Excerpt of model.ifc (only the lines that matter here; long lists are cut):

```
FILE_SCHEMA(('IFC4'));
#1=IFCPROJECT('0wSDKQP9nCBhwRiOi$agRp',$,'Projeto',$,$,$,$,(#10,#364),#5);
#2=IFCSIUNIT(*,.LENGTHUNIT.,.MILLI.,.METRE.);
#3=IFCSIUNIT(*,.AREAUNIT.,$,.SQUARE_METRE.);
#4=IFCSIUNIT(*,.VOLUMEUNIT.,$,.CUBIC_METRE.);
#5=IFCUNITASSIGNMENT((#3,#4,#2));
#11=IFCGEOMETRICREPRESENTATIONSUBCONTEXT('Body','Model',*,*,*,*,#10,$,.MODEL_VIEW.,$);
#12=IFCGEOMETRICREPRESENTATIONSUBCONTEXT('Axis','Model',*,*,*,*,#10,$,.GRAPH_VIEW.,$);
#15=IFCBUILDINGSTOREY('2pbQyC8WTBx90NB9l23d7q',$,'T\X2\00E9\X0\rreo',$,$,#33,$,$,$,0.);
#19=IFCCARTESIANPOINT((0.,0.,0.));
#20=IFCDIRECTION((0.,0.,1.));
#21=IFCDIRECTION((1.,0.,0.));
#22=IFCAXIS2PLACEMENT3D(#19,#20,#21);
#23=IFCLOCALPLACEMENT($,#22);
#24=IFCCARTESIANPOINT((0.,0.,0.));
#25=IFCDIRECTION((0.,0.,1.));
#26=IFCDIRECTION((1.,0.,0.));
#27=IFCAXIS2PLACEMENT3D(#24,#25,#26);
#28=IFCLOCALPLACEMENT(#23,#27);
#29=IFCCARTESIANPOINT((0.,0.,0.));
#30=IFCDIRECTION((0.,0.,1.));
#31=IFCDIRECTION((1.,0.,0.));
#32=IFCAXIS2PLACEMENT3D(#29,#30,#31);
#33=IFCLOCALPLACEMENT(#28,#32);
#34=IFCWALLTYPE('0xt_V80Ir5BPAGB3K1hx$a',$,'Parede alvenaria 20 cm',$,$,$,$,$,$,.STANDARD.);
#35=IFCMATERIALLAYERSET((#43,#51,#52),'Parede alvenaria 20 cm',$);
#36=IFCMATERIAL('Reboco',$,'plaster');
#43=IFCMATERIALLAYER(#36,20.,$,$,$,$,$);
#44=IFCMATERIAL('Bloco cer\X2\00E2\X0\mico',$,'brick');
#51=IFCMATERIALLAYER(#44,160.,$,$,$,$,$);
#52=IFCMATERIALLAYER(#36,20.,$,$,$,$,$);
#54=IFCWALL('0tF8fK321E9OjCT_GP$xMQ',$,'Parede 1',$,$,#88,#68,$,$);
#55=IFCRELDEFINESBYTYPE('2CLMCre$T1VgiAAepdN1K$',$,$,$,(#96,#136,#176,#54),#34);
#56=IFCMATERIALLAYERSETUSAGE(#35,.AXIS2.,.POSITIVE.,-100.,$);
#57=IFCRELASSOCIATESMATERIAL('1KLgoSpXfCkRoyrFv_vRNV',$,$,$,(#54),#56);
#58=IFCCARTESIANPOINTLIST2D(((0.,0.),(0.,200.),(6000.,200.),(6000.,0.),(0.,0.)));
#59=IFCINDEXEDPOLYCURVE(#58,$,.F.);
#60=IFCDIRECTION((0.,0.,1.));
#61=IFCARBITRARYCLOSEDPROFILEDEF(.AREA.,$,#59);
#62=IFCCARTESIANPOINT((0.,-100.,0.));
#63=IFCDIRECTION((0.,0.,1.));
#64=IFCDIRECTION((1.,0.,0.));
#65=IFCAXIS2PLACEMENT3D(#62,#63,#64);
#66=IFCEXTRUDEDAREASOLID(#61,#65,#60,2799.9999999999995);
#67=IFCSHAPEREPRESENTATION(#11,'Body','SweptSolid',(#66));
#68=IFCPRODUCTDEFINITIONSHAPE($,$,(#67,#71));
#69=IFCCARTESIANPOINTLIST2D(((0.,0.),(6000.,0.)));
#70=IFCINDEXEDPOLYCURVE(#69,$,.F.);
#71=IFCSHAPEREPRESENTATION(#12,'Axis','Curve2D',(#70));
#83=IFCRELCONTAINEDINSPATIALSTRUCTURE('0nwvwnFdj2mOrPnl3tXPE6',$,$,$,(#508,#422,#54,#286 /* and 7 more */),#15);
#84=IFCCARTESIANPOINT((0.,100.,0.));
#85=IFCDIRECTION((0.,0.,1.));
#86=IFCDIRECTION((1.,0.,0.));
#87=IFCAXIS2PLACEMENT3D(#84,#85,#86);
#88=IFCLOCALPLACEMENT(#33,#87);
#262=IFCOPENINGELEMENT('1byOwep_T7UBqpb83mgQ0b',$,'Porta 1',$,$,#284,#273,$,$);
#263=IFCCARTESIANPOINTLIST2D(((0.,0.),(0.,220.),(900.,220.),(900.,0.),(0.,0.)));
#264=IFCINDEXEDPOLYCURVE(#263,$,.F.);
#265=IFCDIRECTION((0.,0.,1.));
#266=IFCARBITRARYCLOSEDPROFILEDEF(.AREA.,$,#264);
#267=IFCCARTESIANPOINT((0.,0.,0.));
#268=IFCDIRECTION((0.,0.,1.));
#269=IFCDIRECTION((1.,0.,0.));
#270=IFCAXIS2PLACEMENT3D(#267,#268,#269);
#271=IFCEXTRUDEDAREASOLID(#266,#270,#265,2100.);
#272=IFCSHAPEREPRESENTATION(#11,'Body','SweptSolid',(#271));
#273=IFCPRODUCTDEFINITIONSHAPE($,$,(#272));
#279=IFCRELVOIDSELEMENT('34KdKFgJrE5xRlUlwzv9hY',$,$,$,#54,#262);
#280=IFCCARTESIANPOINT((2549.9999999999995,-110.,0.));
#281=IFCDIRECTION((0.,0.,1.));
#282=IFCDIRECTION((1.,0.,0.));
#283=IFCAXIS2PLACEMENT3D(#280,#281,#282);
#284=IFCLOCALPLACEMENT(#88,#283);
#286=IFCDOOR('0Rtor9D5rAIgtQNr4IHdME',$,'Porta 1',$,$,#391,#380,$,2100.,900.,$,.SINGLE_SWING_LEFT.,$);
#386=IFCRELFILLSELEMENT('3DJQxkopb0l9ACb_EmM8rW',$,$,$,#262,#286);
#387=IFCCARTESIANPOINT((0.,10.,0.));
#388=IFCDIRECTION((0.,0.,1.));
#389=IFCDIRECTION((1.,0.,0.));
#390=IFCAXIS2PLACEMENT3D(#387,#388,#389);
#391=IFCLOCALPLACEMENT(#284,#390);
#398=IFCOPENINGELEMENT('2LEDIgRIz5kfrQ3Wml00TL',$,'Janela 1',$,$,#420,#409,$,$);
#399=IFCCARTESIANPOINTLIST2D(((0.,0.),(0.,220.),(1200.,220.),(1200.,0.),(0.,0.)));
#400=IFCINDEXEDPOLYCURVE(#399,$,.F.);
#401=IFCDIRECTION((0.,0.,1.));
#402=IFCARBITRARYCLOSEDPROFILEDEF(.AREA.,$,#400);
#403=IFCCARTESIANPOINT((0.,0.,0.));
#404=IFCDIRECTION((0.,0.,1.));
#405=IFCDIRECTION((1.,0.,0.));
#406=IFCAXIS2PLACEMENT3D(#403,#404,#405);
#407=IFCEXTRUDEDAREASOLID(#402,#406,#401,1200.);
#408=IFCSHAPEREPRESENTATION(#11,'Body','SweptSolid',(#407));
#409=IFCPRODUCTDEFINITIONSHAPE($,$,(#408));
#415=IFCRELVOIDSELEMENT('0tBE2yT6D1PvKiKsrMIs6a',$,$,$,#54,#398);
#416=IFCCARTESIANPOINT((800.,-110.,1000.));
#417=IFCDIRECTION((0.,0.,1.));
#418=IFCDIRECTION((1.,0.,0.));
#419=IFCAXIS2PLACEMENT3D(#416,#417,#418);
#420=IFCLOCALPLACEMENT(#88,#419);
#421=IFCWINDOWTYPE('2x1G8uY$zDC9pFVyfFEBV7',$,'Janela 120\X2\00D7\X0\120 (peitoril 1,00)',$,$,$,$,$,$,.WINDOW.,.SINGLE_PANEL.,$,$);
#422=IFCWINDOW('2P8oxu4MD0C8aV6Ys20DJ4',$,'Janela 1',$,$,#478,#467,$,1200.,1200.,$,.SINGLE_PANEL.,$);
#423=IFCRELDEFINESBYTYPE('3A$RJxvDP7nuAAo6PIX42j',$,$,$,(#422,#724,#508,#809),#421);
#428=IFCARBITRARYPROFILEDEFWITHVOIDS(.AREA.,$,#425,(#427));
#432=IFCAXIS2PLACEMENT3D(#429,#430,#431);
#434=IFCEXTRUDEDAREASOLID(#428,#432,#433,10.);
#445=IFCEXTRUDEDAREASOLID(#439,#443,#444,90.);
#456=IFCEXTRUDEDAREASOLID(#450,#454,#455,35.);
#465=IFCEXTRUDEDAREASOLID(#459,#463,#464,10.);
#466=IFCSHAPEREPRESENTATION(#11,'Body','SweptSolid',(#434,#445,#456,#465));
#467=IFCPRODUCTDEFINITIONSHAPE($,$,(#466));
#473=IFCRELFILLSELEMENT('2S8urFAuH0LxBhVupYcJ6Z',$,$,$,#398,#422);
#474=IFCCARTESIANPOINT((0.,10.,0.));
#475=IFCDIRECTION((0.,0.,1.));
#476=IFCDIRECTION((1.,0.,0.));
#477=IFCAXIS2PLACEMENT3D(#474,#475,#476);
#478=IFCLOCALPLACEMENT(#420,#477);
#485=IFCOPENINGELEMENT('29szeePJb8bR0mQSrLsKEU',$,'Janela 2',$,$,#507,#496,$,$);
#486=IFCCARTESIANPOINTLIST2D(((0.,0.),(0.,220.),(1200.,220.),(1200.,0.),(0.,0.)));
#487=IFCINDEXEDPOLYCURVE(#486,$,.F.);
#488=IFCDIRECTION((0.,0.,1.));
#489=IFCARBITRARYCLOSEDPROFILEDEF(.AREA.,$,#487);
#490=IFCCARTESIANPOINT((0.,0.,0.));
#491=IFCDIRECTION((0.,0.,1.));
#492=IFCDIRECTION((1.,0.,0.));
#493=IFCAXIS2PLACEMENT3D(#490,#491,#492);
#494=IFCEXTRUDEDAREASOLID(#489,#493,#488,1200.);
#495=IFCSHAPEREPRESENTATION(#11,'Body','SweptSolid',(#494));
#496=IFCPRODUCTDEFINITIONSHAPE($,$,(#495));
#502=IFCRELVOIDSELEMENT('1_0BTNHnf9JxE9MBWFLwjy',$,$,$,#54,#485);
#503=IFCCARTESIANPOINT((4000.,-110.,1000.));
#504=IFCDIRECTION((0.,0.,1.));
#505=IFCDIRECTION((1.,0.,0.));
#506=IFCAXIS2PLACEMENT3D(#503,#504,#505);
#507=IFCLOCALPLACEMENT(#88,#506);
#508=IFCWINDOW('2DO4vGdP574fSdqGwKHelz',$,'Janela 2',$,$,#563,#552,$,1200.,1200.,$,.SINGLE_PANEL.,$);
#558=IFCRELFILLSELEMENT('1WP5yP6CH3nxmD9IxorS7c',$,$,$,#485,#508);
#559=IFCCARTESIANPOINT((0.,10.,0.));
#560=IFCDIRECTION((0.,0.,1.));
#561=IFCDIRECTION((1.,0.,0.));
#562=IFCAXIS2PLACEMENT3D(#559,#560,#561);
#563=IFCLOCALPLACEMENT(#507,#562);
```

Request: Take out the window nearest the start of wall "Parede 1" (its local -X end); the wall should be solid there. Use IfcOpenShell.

```python
import ifcopenshell
import ifcopenshell.api.feature
import ifcopenshell.api.root
import ifcopenshell.geom
import ifcopenshell.util.shape

model = ifcopenshell.open("model.ifc")
settings = ifcopenshell.geom.settings()


def volume(element):
    """Net volume in cubic metres, openings subtracted."""
    shape = ifcopenshell.geom.create_shape(settings, element)
    return ifcopenshell.util.shape.get_volume(shape.geometry)


window = model.by_guid("2P8oxu4MD0C8aV6Ys20DJ4")
opening = window.FillsVoids[0].RelatingOpeningElement
wall = opening.VoidsElements[0].RelatingBuildingElement
before = volume(wall)

ifcopenshell.api.root.remove_product(model, product=window)
ifcopenshell.api.feature.remove_feature(model, feature=opening)

after = volume(wall)

print(f"wall volume {before:.3f} -> {after:.3f} m3")

model.write("model-out.ifc")
```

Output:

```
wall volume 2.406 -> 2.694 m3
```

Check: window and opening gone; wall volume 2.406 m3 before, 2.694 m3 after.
